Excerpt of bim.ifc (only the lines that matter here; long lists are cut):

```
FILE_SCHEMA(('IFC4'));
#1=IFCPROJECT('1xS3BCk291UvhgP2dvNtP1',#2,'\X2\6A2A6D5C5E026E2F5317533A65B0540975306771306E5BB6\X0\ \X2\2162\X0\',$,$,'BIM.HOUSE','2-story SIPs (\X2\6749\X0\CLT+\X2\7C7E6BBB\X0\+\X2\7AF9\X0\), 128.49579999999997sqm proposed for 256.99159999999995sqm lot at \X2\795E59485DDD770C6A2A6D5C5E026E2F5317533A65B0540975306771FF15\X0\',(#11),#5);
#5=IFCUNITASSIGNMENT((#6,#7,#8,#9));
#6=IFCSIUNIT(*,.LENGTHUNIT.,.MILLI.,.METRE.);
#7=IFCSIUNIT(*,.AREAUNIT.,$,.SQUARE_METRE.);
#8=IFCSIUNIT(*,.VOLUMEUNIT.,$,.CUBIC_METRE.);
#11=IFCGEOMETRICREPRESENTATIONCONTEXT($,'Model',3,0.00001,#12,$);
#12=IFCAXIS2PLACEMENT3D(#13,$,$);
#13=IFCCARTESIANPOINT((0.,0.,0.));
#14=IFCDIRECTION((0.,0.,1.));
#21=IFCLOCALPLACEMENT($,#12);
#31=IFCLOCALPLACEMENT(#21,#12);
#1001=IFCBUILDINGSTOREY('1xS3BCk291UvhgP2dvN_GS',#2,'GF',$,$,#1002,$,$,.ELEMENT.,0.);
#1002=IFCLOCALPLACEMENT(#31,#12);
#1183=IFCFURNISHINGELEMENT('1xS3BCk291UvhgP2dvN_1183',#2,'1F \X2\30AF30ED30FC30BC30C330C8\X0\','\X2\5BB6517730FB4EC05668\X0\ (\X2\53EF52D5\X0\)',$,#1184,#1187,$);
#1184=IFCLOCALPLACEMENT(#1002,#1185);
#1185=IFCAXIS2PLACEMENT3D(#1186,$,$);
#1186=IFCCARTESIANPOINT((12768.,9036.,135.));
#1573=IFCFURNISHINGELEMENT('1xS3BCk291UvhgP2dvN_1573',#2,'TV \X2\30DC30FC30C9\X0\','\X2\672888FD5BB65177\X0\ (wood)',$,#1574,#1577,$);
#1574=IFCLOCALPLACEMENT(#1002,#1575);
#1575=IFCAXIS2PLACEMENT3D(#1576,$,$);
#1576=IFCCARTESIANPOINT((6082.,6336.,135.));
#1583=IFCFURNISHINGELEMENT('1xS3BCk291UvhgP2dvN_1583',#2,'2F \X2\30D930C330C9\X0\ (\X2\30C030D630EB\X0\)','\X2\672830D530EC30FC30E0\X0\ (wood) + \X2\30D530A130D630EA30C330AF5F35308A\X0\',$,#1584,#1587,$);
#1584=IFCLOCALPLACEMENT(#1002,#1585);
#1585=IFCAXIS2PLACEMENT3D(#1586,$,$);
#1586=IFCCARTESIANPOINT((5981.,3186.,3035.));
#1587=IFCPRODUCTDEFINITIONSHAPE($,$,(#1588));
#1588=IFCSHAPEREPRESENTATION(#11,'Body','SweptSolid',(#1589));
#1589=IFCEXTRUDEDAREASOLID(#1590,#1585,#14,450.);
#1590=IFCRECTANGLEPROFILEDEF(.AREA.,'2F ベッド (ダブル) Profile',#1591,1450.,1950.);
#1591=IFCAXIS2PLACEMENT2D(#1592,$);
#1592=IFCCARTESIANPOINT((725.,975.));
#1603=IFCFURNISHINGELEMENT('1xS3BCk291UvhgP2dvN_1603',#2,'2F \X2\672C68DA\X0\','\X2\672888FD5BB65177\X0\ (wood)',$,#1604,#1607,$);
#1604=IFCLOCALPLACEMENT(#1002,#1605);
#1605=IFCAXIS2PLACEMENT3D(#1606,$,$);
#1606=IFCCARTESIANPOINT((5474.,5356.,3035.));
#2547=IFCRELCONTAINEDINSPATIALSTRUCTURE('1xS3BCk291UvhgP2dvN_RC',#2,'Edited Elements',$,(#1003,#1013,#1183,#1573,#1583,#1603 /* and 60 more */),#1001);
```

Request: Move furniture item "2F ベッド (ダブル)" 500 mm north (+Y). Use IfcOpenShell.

```python
import ifcopenshell
import ifcopenshell.api.geometry
import ifcopenshell.util.placement

model = ifcopenshell.open("bim.ifc")

item = model.by_guid("1xS3BCk291UvhgP2dvN_1583")
matrix = ifcopenshell.util.placement.get_local_placement(item.ObjectPlacement)
matrix[1, 3] += 500.0
ifcopenshell.api.geometry.edit_object_placement(model, product=item, matrix=matrix, is_si=False)

print(ifcopenshell.util.placement.get_local_placement(item.ObjectPlacement).round(3) + 0.0)

model.write("bim_rev.ifc")
```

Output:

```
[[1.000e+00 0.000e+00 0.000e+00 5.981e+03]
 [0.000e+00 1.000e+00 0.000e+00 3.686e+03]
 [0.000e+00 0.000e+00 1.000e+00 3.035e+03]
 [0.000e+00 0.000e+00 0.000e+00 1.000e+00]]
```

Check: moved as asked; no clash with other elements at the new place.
